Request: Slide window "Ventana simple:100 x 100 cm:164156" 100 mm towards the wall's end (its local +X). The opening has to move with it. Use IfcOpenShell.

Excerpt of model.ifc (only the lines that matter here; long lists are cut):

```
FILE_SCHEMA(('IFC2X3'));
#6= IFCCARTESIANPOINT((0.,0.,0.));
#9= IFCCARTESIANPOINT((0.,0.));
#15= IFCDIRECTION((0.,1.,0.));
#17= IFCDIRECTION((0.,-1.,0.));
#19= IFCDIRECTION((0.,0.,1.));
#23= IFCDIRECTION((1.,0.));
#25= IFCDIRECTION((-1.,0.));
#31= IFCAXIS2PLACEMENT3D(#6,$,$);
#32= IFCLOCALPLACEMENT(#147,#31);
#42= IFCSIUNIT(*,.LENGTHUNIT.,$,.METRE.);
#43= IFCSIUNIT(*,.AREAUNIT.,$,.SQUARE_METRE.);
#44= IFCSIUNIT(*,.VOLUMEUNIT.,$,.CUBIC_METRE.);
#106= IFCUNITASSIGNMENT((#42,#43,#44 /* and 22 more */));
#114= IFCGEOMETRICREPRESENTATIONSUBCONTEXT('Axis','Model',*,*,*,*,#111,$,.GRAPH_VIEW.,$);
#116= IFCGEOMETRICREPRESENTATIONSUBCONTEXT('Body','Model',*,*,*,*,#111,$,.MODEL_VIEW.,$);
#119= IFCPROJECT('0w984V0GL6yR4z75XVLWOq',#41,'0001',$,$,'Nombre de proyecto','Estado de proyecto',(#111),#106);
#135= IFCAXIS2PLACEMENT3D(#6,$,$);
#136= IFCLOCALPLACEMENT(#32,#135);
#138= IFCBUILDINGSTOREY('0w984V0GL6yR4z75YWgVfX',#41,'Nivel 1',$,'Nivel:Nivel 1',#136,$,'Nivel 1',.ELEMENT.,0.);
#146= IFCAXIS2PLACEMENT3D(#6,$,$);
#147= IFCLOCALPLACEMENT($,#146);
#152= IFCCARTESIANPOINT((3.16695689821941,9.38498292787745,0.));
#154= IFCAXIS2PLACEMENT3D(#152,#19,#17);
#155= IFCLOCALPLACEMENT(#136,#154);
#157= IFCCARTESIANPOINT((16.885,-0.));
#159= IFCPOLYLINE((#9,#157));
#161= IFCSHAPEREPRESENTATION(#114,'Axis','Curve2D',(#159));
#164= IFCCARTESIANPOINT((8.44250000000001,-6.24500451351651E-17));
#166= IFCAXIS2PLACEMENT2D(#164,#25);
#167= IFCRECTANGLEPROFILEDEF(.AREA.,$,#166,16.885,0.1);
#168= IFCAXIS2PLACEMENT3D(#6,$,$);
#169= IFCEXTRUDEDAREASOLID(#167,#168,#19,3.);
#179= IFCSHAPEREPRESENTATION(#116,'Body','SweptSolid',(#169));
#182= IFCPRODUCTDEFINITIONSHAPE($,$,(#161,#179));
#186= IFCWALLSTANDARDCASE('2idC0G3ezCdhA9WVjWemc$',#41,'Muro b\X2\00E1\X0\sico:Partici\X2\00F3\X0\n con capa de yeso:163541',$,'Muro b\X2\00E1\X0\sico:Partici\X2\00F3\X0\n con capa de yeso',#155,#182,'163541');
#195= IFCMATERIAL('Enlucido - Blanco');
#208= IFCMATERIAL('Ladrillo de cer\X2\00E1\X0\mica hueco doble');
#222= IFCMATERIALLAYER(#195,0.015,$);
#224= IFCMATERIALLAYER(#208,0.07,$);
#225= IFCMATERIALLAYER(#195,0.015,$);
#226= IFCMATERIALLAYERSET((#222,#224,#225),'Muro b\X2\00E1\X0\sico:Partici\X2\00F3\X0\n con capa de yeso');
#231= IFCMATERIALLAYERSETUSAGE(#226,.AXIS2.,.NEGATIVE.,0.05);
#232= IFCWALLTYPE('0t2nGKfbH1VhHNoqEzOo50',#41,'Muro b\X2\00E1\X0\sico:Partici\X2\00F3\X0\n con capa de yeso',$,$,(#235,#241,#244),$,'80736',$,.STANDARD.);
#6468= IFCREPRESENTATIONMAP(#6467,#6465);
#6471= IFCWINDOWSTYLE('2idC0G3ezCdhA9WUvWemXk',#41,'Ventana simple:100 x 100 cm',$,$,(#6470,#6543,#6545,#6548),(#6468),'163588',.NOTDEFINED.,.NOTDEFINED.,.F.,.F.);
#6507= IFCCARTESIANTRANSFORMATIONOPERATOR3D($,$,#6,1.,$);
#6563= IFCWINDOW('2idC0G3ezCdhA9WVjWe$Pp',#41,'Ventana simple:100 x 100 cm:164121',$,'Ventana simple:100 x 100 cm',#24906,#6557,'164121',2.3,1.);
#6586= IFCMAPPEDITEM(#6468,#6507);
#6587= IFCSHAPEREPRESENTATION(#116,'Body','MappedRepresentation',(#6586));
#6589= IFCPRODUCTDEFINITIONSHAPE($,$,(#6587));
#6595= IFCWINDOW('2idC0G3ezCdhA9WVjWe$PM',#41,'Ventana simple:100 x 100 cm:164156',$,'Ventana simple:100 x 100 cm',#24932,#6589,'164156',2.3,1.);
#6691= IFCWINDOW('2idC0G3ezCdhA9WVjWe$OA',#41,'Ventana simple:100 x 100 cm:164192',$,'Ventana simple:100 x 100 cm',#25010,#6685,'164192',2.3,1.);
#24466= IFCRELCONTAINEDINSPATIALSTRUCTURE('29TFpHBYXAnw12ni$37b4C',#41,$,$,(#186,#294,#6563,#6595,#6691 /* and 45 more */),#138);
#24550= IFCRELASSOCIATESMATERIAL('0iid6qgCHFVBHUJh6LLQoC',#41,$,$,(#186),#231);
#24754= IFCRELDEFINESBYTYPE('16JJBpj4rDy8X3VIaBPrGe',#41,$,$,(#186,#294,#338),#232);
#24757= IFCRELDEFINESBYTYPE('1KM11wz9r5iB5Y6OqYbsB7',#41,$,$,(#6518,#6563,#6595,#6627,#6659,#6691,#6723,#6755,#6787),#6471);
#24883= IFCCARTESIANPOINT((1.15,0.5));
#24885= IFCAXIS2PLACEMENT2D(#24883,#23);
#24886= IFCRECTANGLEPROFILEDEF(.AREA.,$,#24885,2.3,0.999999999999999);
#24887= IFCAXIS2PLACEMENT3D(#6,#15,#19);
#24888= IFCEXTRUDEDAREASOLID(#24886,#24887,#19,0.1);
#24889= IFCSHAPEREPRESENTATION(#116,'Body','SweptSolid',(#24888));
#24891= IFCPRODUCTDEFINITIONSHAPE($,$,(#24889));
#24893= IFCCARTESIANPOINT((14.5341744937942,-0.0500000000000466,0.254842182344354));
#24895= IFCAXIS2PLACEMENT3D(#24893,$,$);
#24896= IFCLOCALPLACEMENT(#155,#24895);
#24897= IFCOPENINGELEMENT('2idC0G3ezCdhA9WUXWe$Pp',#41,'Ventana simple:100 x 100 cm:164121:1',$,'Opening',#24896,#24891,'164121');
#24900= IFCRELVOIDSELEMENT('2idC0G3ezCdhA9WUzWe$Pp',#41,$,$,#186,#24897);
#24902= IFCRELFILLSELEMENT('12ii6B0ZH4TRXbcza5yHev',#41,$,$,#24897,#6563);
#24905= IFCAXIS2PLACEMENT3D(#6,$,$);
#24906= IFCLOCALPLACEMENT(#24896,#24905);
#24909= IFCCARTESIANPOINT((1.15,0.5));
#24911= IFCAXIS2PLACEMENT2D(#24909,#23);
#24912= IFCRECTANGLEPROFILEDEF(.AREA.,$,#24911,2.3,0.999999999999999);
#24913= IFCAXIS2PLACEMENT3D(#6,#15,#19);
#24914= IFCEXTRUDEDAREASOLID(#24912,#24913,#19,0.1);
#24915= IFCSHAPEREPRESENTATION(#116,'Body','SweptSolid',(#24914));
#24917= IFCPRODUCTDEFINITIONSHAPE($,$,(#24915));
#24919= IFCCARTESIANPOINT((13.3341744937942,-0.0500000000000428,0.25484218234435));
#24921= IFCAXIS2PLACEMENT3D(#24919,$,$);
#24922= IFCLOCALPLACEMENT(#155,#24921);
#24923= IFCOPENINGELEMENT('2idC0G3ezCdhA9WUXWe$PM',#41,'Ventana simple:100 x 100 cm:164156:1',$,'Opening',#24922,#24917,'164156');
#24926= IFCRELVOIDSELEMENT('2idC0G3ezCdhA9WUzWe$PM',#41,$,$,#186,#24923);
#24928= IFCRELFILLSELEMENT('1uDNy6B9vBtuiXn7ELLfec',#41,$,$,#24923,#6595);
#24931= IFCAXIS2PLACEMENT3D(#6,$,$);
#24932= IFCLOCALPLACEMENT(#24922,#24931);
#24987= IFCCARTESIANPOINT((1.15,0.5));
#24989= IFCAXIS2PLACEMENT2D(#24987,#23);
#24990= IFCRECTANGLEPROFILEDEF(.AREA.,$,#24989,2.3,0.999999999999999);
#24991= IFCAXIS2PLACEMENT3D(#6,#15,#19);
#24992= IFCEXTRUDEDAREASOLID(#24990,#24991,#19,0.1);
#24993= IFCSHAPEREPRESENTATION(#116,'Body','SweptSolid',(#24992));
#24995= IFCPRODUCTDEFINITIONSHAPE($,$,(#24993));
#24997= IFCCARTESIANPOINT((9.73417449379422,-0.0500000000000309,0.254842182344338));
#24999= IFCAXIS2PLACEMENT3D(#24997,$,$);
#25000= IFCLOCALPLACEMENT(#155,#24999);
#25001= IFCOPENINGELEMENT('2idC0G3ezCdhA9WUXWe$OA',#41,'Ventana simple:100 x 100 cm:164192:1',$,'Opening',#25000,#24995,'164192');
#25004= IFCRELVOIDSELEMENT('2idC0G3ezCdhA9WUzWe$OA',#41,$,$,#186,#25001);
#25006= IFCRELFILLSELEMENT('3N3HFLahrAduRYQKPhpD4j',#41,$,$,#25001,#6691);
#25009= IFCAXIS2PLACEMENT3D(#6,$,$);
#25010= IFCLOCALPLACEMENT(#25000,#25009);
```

```python
import ifcopenshell
import ifcopenshell.api.geometry
import ifcopenshell.util.placement
import ifcopenshell.util.unit

model = ifcopenshell.open("model.ifc")
unit_scale = ifcopenshell.util.unit.calculate_unit_scale(model)

window = model.by_id(6595)
opening = window.FillsVoids[0].RelatingOpeningElement
wall = opening.VoidsElements[0].RelatingBuildingElement

wall_matrix = ifcopenshell.util.placement.get_local_placement(wall.ObjectPlacement)
shift = wall_matrix[:3, 0] * 0.1 / unit_scale
before = ifcopenshell.util.placement.get_local_placement(window.ObjectPlacement)[:3, 3].copy()

# The window is placed relative to its opening, so it follows when the opening moves.
matrix = ifcopenshell.util.placement.get_local_placement(opening.ObjectPlacement)
matrix[:3, 3] += shift
ifcopenshell.api.geometry.edit_object_placement(
    model, product=opening, matrix=matrix, is_si=False, should_transform_children=True
)

after = ifcopenshell.util.placement.get_local_placement(window.ObjectPlacement)[:3, 3]
print("window moved by", (after - before).round(3) + 0.0)

model.write("model_v2.ifc")
```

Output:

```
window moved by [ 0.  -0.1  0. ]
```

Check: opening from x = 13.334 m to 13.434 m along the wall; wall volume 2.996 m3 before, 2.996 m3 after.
